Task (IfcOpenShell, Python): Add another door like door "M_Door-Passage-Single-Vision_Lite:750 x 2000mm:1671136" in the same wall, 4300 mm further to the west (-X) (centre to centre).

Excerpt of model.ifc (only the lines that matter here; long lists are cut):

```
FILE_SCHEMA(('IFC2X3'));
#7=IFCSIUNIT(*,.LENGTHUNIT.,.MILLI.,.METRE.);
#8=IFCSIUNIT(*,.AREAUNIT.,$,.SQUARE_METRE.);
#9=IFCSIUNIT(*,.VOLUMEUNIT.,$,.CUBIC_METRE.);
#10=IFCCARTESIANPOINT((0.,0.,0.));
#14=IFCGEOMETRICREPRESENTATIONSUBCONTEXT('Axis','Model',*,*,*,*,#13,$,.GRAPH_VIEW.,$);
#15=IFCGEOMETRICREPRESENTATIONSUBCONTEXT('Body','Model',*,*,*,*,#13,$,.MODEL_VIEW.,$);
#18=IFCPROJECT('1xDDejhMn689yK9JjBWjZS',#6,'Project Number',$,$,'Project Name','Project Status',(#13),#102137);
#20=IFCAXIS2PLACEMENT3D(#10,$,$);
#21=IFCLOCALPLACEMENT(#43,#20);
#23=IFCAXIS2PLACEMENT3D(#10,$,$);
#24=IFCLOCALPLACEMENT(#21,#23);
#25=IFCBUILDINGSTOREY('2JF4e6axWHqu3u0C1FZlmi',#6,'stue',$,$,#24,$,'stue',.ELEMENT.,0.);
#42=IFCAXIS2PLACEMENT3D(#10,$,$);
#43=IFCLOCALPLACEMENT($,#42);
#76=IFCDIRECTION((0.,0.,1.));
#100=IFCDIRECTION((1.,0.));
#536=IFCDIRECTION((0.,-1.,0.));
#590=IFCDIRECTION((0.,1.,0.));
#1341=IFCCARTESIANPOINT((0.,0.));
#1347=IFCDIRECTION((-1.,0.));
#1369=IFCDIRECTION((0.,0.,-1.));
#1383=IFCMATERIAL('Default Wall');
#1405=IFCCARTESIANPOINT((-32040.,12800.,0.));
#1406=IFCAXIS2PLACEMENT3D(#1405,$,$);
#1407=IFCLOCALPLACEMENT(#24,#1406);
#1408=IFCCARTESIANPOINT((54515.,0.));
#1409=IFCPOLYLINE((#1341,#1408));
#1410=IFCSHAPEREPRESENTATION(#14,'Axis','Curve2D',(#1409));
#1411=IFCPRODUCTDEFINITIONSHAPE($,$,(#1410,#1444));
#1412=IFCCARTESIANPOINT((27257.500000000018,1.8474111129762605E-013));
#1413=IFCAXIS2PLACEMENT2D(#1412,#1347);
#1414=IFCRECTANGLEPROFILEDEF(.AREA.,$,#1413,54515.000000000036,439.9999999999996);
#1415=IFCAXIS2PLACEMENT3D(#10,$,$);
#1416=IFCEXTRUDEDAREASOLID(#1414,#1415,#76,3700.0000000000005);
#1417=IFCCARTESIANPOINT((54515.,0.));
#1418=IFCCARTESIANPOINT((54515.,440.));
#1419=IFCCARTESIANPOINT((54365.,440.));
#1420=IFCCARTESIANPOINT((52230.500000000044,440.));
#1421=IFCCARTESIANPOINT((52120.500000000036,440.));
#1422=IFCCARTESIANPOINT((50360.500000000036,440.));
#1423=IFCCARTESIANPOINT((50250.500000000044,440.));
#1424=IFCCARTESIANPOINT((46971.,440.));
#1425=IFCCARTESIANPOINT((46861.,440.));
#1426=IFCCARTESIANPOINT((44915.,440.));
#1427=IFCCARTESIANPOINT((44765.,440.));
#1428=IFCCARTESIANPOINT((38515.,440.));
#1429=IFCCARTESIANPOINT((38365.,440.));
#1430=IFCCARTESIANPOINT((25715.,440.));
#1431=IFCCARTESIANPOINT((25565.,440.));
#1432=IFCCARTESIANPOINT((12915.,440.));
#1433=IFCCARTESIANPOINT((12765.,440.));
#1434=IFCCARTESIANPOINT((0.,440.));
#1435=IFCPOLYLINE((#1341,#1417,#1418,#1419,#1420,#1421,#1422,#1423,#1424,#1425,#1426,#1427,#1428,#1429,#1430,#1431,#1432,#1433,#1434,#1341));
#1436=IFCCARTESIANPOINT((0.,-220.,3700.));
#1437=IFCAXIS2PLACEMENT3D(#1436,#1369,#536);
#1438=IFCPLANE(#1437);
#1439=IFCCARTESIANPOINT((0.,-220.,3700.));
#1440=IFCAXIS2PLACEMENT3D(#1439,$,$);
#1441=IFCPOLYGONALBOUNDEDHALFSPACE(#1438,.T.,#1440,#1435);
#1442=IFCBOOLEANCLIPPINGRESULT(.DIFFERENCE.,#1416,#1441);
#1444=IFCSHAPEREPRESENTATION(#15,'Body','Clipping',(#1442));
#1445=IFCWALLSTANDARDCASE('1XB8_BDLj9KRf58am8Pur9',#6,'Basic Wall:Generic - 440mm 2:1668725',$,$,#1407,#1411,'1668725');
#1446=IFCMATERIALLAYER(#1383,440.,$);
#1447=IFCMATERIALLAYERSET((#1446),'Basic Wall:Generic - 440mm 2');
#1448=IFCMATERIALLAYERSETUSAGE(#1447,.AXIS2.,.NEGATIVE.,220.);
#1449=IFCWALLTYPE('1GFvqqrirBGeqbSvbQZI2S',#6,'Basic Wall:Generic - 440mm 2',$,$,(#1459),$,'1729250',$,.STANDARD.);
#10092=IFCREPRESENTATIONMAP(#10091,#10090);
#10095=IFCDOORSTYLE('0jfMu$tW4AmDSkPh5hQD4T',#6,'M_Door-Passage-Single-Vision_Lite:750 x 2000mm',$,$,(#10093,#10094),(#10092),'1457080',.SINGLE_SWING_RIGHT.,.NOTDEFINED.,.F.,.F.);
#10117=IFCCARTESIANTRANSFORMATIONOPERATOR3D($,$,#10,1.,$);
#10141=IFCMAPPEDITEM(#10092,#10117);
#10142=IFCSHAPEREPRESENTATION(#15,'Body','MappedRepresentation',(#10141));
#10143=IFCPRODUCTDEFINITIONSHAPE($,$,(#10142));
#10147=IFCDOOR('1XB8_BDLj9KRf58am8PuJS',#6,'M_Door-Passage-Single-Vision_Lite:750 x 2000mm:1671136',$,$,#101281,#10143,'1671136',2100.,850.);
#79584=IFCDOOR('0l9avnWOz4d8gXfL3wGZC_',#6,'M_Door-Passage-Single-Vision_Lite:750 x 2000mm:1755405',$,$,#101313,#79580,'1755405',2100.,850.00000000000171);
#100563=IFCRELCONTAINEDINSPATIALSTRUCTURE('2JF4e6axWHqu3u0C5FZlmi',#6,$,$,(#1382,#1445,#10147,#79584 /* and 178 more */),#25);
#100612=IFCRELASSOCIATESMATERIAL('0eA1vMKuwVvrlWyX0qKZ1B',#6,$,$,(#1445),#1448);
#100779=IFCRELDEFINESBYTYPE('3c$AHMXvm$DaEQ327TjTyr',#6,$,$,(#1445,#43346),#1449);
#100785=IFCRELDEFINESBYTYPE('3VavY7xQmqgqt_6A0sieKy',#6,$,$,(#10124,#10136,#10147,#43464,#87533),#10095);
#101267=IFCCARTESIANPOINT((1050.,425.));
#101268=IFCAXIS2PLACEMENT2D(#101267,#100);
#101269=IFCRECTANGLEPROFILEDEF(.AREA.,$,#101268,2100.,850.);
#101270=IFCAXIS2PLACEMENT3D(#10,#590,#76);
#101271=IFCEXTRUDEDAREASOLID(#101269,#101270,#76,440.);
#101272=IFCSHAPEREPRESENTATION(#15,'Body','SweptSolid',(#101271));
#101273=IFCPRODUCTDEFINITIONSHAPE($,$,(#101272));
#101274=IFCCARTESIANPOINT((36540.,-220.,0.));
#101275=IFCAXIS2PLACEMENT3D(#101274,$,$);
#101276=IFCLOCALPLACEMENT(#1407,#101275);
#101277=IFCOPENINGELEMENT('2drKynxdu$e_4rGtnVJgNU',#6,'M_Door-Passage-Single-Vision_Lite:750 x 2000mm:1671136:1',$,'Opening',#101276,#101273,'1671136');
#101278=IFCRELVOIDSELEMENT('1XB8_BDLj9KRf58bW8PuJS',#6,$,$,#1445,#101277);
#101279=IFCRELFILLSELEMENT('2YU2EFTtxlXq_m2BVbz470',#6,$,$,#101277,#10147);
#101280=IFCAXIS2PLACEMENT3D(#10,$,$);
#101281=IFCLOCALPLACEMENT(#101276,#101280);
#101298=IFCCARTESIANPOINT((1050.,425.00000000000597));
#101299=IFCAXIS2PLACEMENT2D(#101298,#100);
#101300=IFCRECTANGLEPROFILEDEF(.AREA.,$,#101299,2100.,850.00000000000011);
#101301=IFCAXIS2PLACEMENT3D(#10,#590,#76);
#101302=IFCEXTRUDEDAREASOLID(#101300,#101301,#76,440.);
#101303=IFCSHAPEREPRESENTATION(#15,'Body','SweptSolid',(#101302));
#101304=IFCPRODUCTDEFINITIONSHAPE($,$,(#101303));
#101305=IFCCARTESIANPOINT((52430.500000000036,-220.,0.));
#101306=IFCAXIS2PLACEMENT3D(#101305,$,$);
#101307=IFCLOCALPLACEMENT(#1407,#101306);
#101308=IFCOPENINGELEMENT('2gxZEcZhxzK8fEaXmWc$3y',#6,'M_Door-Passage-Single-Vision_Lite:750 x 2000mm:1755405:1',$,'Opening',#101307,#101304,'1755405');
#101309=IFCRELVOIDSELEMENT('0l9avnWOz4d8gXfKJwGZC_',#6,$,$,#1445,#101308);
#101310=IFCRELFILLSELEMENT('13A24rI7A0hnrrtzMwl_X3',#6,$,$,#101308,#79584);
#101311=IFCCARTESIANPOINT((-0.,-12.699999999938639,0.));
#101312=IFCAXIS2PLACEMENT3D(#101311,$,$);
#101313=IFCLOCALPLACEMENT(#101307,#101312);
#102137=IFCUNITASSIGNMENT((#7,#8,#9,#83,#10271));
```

```python
import ifcopenshell
import ifcopenshell.api.feature
import ifcopenshell.api.geometry
import ifcopenshell.api.root
import ifcopenshell.geom
import ifcopenshell.util.element
import ifcopenshell.util.placement
import ifcopenshell.util.shape

model = ifcopenshell.open("model.ifc")
settings = ifcopenshell.geom.settings()


def volume(element):
    """Net volume in cubic metres, openings subtracted."""
    shape = ifcopenshell.geom.create_shape(settings, element)
    return ifcopenshell.util.shape.get_volume(shape.geometry)


def reuse_history(source, copy):
    """copy_class also copies each property set's owner history, people and application; keep the originals."""
    for rel in copy.IsDefinedBy:
        if rel.is_a("IfcRelDefinesByProperties") and (history := rel.RelatingPropertyDefinition.OwnerHistory):
            rel.RelatingPropertyDefinition.OwnerHistory = source.OwnerHistory
            ifcopenshell.util.element.remove_deep2(model, history)


door = model.by_guid("1XB8_BDLj9KRf58am8PuJS")
opening = door.FillsVoids[0].RelatingOpeningElement
wall = opening.VoidsElements[0].RelatingBuildingElement
before = volume(wall)
shift = ifcopenshell.util.placement.get_local_placement(wall.ObjectPlacement)[:3, 0] * -4300.0

# copy_class copies the void relationship, type, container and properties, but no geometry.
new_opening = ifcopenshell.api.root.copy_class(model, product=opening)
new_opening.Representation = ifcopenshell.util.element.copy_deep(
    model, opening.Representation, exclude=["IfcGeometricRepresentationContext", "IfcRepresentationMap"]
)
new_opening.Name = "M_Door-Passage-Single-Vision_Lite:750 x 2000mm"
new_opening.Tag = None
new_door = ifcopenshell.api.root.copy_class(model, product=door)
new_door.Representation = ifcopenshell.util.element.copy_deep(
    model, door.Representation, exclude=["IfcGeometricRepresentationContext", "IfcRepresentationMap"]
)
new_door.Name = "M_Door-Passage-Single-Vision_Lite:750 x 2000mm"
new_door.Tag = None
reuse_history(door, new_door)
fills = ifcopenshell.api.feature.add_filling(model, opening=new_opening, element=new_door)
fills.OwnerHistory = new_door.OwnerHistory  # required in IFC2X3

for old, new in ((opening, new_opening), (door, new_door)):
    matrix = ifcopenshell.util.placement.get_local_placement(old.ObjectPlacement)
    matrix[:3, 3] += shift
    ifcopenshell.api.geometry.edit_object_placement(model, product=new, matrix=matrix, is_si=False)

after = volume(wall)

print(f"wall volume {before:.3f} -> {after:.3f} m3")

model.write("model_edited.ifc")
```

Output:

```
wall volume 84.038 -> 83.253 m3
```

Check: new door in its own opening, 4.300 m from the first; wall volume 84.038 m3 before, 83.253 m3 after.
